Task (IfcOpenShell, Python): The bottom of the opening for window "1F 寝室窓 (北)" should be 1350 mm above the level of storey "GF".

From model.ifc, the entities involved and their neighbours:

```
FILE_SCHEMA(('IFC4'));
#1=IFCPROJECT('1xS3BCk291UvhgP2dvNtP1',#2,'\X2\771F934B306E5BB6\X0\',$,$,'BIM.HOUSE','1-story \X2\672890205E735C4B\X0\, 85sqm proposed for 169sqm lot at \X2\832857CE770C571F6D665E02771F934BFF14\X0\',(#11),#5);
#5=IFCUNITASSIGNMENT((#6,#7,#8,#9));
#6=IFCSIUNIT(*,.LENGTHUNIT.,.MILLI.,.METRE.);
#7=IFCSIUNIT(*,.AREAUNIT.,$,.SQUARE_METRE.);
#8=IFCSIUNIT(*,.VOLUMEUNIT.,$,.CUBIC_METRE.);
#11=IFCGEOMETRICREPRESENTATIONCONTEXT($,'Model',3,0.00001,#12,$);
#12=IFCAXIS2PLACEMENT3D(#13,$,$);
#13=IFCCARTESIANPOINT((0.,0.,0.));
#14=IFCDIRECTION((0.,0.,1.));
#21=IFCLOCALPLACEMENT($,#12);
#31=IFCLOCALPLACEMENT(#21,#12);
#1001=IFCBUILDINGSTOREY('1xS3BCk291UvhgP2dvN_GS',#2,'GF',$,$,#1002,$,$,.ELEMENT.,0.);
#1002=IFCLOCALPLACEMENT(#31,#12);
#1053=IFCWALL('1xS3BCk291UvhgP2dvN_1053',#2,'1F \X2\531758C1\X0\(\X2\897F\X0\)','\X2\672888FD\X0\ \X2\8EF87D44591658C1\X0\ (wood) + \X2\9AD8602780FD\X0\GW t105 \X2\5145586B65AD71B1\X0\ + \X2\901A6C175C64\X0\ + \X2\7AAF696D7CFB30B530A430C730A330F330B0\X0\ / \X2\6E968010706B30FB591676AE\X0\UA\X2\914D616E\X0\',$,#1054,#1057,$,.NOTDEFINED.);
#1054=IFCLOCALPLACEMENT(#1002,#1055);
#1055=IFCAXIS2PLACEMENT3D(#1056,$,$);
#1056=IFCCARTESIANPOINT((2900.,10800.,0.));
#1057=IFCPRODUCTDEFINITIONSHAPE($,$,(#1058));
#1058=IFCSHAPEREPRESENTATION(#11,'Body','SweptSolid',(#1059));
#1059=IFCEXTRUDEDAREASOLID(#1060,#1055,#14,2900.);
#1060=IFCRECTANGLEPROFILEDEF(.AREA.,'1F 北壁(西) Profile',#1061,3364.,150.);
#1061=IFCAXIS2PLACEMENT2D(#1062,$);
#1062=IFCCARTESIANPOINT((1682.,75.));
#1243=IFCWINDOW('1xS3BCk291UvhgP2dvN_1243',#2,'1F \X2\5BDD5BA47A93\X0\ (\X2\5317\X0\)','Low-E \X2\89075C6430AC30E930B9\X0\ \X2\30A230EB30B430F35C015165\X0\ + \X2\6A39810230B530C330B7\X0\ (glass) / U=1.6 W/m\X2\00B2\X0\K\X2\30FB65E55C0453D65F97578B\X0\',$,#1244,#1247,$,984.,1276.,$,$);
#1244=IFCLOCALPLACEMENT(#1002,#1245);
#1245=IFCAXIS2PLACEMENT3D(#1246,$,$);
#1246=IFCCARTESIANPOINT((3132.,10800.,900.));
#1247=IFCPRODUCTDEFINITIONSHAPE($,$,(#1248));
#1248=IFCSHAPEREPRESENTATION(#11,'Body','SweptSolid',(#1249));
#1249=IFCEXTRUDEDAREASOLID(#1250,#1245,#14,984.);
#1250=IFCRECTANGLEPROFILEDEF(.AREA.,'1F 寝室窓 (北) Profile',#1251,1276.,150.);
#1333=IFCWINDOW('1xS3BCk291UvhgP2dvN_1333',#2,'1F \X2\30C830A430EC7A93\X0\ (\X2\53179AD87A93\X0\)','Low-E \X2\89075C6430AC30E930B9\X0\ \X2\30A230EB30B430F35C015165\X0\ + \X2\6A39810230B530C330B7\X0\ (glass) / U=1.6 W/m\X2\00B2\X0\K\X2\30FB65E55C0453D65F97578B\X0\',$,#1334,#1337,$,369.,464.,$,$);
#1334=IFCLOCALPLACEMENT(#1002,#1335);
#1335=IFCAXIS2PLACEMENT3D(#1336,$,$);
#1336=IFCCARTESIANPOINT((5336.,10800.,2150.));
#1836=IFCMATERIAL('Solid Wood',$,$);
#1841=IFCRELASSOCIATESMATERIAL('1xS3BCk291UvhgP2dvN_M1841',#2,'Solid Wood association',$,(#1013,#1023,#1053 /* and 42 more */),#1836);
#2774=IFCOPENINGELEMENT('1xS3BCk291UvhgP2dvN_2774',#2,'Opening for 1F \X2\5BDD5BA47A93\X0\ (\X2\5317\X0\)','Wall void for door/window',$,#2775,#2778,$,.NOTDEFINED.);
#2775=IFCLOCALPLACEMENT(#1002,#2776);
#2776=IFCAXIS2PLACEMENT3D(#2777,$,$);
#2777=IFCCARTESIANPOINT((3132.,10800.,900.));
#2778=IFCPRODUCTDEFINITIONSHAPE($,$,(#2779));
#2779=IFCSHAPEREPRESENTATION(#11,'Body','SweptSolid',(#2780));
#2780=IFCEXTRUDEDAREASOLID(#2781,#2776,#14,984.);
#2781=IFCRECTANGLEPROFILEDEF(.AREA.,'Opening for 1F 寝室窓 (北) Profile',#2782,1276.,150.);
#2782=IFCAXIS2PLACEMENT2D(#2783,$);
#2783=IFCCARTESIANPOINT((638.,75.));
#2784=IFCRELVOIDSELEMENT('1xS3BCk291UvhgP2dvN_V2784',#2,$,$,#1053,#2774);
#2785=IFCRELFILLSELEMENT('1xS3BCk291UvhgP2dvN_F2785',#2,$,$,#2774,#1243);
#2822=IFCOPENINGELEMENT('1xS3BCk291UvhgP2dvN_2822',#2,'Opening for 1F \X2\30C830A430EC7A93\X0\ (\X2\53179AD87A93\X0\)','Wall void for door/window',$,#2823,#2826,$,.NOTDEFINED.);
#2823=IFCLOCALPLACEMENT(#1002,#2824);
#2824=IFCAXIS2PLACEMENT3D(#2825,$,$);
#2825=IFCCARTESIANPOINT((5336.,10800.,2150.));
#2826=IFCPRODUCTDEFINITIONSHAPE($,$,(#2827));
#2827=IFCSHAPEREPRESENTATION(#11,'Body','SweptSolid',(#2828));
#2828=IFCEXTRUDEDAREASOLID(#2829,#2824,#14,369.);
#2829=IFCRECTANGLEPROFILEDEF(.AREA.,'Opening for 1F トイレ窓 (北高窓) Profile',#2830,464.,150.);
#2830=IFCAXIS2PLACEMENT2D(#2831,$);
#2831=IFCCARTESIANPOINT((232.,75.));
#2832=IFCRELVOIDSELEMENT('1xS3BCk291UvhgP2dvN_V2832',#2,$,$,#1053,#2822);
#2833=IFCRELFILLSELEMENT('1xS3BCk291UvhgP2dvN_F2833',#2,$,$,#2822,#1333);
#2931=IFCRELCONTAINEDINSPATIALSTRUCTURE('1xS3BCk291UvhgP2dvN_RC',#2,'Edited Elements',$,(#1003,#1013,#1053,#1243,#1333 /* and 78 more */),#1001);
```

```python
import numpy as np
import ifcopenshell
import ifcopenshell.api.geometry
import ifcopenshell.geom
import ifcopenshell.util.element
import ifcopenshell.util.placement
import ifcopenshell.util.shape
import ifcopenshell.util.unit

model = ifcopenshell.open("model.ifc")
unit_scale = ifcopenshell.util.unit.calculate_unit_scale(model)

window = model.by_guid("1xS3BCk291UvhgP2dvN_1243")
opening = window.FillsVoids[0].RelatingOpeningElement
storey = ifcopenshell.util.element.get_container(window, ifc_class="IfcBuildingStorey")
level = ifcopenshell.util.placement.get_local_placement(storey.ObjectPlacement)[2, 3]

# The opening's origin need not be at the sill, so measure its lowest point.
shape = ifcopenshell.geom.create_shape(ifcopenshell.geom.settings(), opening)
bottom = ifcopenshell.util.shape.get_shape_bottom_elevation(shape, shape.geometry) / unit_scale
dz = level + 1.35 / unit_scale - bottom

shift = np.array([0.0, 0.0, dz])
# The window is not placed relative to its opening, so move both.
for product in (opening, window):
    matrix = ifcopenshell.util.placement.get_local_placement(product.ObjectPlacement)
    matrix[:3, 3] += shift
    ifcopenshell.api.geometry.edit_object_placement(model, product=product, matrix=matrix, is_si=False)

print(f"moved by {dz * unit_scale:+.3f} m")

model.write("model-out.ifc")
```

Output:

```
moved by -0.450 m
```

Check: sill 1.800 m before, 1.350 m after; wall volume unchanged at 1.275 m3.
